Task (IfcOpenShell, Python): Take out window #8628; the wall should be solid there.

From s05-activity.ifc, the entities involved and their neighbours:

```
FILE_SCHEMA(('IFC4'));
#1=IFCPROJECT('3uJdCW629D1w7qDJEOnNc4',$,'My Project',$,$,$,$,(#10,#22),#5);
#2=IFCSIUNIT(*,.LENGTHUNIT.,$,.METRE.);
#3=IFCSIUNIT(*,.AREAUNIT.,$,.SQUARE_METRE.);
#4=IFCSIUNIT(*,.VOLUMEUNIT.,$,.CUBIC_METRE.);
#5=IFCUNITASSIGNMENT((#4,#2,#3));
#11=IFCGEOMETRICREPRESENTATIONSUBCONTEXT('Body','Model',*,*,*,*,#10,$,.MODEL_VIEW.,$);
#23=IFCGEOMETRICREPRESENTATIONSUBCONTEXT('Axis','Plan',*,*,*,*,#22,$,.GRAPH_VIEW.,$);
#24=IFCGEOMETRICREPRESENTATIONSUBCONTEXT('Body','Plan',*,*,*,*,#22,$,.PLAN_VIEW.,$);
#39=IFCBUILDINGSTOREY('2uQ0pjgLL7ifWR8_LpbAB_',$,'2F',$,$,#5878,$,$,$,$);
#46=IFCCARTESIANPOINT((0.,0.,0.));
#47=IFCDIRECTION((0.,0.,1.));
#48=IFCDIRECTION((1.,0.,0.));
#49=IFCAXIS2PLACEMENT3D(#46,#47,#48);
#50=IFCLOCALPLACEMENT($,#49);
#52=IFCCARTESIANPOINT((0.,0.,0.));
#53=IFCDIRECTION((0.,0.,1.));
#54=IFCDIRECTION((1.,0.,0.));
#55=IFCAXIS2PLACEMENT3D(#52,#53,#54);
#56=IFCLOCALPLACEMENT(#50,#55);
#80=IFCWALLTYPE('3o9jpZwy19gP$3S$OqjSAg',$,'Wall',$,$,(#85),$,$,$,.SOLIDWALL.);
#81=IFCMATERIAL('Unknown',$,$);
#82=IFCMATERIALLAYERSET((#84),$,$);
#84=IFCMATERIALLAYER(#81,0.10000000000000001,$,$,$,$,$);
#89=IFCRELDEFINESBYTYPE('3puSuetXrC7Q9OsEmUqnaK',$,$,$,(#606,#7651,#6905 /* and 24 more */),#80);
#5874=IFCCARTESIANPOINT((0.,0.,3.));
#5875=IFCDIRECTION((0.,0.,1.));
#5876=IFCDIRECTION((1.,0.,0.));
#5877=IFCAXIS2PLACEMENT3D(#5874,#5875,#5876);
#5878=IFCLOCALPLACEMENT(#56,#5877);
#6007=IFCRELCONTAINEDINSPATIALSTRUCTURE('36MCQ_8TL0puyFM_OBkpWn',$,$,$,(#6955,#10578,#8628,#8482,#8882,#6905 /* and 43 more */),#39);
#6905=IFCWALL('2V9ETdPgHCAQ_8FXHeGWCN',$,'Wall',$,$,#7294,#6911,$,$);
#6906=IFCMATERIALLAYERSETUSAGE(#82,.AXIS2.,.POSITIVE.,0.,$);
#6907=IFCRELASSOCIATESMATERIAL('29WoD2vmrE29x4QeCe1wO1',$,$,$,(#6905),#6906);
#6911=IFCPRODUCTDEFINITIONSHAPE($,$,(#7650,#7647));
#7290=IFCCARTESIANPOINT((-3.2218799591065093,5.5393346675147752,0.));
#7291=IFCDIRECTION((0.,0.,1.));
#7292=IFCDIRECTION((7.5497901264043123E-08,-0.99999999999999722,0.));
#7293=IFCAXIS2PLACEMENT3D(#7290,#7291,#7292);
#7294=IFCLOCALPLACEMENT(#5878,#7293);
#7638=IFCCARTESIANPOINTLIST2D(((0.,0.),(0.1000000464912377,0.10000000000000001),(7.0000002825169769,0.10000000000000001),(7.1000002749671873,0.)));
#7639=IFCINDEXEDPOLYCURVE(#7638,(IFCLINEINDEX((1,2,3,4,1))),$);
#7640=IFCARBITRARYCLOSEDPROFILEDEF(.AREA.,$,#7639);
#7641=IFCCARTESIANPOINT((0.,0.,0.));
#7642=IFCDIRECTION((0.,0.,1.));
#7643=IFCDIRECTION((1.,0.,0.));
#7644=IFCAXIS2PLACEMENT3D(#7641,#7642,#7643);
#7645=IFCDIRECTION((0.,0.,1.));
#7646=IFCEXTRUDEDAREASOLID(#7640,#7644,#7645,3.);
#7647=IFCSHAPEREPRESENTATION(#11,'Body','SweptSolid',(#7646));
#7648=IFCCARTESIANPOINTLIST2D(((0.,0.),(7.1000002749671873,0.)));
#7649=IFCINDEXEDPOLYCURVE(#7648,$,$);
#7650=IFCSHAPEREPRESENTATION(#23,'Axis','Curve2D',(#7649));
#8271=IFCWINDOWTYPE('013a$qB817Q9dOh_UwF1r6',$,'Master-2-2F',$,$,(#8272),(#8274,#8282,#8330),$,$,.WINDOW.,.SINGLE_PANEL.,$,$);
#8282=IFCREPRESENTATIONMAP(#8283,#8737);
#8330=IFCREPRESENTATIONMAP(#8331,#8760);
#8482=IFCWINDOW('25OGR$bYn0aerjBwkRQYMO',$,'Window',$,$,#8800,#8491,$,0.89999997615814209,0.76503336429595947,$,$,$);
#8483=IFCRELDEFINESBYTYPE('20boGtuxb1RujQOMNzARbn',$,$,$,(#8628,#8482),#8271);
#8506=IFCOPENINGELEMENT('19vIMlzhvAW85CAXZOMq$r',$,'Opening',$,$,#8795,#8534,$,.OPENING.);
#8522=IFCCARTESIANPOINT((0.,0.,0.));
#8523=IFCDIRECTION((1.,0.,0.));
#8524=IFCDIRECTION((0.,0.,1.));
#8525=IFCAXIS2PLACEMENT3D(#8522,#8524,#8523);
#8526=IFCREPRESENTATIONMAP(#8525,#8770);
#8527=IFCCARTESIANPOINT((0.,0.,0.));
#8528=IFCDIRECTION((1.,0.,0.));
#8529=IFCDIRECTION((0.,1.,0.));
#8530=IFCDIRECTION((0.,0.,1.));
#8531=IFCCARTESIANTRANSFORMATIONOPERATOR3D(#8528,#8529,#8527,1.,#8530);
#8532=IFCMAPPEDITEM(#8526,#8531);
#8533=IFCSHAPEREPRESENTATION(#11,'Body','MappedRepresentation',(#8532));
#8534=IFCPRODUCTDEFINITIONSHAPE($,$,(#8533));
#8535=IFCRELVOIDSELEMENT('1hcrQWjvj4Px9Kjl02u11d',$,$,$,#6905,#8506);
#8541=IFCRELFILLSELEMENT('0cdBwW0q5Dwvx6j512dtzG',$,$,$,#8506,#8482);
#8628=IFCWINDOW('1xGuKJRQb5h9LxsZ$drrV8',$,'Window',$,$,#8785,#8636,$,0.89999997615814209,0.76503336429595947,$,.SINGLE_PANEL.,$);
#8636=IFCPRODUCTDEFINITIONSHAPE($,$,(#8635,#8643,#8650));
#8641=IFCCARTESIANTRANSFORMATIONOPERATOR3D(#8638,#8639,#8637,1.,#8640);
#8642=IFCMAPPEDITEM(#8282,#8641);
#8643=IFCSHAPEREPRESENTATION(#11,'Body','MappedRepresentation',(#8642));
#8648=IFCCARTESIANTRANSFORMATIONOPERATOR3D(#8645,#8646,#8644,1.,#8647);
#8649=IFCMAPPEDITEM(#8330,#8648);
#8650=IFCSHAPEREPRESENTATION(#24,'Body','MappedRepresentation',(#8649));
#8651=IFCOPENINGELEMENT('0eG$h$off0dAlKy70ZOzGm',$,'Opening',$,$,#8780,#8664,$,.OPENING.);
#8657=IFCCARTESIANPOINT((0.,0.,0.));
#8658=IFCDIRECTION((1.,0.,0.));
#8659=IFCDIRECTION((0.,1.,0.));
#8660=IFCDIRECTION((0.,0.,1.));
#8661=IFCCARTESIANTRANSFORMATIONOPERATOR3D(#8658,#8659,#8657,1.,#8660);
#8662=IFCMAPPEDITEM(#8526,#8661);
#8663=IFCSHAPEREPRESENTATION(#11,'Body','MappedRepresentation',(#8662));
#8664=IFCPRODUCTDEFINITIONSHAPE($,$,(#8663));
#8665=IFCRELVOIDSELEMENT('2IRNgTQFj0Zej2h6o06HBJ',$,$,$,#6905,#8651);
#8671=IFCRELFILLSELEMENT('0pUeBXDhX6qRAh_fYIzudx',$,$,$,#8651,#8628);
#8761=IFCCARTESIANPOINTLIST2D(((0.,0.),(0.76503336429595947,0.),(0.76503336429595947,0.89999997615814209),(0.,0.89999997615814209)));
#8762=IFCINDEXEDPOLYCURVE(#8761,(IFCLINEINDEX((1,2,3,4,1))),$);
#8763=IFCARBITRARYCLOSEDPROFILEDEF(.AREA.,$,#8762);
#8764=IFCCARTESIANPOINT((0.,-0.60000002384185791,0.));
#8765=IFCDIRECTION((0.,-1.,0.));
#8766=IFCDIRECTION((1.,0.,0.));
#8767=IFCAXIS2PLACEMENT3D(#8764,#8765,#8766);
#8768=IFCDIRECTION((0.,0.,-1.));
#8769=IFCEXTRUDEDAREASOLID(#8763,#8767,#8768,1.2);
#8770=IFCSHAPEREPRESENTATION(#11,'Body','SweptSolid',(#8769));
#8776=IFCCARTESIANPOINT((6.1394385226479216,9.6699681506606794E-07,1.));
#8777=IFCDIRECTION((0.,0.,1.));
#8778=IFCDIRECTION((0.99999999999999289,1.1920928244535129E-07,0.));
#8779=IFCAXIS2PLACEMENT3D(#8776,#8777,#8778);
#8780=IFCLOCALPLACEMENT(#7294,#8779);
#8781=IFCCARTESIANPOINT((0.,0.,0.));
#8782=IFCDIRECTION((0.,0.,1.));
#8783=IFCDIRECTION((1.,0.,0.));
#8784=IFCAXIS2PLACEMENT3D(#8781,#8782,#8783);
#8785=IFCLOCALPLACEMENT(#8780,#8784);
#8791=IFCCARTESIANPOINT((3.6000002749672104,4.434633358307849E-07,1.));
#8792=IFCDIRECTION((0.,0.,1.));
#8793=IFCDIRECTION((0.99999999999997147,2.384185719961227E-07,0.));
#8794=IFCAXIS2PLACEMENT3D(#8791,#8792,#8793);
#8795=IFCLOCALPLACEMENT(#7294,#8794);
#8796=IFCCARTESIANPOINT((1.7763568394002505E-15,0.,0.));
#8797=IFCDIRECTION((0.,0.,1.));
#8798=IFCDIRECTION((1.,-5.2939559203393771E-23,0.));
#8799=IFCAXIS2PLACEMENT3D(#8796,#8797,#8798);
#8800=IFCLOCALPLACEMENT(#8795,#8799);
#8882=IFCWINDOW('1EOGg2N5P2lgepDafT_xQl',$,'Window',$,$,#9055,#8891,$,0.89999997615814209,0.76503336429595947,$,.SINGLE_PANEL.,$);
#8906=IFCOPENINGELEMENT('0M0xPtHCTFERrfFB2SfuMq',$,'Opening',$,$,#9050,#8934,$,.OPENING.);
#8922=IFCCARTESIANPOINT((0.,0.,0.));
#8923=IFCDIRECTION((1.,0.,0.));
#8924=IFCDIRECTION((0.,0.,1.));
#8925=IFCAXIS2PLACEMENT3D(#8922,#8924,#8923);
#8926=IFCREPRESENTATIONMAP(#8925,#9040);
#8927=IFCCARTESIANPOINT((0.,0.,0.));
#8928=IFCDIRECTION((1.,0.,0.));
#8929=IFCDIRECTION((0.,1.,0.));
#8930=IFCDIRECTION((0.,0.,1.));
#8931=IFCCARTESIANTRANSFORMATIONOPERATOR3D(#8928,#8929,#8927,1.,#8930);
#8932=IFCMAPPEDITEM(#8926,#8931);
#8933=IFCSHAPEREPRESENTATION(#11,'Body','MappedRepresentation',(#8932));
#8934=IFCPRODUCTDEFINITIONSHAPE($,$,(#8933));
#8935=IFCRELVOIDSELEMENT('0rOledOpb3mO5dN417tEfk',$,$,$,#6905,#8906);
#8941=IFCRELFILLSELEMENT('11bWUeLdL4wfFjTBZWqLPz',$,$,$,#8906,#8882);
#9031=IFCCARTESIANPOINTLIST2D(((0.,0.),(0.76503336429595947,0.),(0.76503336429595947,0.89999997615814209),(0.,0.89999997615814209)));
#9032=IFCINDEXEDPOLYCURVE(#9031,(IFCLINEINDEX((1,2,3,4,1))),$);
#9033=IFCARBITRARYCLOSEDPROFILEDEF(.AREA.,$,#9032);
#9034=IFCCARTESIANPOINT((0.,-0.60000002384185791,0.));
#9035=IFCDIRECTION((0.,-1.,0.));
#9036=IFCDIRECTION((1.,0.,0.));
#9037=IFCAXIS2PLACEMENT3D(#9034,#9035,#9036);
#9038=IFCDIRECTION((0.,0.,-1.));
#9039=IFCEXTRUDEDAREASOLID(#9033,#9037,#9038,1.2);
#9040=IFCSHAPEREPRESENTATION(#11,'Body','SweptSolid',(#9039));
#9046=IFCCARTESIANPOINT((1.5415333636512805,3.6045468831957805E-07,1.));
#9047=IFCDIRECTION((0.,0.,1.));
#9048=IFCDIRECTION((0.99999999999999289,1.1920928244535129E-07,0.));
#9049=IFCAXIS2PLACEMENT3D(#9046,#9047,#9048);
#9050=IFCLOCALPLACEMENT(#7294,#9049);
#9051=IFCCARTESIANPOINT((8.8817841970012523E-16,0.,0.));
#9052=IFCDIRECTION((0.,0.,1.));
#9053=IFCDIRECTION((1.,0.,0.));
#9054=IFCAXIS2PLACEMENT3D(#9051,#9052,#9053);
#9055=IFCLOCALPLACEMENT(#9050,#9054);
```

```python
import ifcopenshell
import ifcopenshell.api.feature
import ifcopenshell.api.root
import ifcopenshell.geom
import ifcopenshell.util.shape

model = ifcopenshell.open("s05-activity.ifc")
settings = ifcopenshell.geom.settings()


def volume(element):
    """Net volume in cubic metres, openings subtracted."""
    shape = ifcopenshell.geom.create_shape(settings, element)
    return ifcopenshell.util.shape.get_volume(shape.geometry)


window = model.by_id(8628)
opening = window.FillsVoids[0].RelatingOpeningElement
wall = opening.VoidsElements[0].RelatingBuildingElement
before = volume(wall)

ifcopenshell.api.root.remove_product(model, product=window)
ifcopenshell.api.feature.remove_feature(model, feature=opening)

after = volume(wall)

print(f"wall volume {before:.3f} -> {after:.3f} m3")

model.write("s05-activity_v2.ifc")
```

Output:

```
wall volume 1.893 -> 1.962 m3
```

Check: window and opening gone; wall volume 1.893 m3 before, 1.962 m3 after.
